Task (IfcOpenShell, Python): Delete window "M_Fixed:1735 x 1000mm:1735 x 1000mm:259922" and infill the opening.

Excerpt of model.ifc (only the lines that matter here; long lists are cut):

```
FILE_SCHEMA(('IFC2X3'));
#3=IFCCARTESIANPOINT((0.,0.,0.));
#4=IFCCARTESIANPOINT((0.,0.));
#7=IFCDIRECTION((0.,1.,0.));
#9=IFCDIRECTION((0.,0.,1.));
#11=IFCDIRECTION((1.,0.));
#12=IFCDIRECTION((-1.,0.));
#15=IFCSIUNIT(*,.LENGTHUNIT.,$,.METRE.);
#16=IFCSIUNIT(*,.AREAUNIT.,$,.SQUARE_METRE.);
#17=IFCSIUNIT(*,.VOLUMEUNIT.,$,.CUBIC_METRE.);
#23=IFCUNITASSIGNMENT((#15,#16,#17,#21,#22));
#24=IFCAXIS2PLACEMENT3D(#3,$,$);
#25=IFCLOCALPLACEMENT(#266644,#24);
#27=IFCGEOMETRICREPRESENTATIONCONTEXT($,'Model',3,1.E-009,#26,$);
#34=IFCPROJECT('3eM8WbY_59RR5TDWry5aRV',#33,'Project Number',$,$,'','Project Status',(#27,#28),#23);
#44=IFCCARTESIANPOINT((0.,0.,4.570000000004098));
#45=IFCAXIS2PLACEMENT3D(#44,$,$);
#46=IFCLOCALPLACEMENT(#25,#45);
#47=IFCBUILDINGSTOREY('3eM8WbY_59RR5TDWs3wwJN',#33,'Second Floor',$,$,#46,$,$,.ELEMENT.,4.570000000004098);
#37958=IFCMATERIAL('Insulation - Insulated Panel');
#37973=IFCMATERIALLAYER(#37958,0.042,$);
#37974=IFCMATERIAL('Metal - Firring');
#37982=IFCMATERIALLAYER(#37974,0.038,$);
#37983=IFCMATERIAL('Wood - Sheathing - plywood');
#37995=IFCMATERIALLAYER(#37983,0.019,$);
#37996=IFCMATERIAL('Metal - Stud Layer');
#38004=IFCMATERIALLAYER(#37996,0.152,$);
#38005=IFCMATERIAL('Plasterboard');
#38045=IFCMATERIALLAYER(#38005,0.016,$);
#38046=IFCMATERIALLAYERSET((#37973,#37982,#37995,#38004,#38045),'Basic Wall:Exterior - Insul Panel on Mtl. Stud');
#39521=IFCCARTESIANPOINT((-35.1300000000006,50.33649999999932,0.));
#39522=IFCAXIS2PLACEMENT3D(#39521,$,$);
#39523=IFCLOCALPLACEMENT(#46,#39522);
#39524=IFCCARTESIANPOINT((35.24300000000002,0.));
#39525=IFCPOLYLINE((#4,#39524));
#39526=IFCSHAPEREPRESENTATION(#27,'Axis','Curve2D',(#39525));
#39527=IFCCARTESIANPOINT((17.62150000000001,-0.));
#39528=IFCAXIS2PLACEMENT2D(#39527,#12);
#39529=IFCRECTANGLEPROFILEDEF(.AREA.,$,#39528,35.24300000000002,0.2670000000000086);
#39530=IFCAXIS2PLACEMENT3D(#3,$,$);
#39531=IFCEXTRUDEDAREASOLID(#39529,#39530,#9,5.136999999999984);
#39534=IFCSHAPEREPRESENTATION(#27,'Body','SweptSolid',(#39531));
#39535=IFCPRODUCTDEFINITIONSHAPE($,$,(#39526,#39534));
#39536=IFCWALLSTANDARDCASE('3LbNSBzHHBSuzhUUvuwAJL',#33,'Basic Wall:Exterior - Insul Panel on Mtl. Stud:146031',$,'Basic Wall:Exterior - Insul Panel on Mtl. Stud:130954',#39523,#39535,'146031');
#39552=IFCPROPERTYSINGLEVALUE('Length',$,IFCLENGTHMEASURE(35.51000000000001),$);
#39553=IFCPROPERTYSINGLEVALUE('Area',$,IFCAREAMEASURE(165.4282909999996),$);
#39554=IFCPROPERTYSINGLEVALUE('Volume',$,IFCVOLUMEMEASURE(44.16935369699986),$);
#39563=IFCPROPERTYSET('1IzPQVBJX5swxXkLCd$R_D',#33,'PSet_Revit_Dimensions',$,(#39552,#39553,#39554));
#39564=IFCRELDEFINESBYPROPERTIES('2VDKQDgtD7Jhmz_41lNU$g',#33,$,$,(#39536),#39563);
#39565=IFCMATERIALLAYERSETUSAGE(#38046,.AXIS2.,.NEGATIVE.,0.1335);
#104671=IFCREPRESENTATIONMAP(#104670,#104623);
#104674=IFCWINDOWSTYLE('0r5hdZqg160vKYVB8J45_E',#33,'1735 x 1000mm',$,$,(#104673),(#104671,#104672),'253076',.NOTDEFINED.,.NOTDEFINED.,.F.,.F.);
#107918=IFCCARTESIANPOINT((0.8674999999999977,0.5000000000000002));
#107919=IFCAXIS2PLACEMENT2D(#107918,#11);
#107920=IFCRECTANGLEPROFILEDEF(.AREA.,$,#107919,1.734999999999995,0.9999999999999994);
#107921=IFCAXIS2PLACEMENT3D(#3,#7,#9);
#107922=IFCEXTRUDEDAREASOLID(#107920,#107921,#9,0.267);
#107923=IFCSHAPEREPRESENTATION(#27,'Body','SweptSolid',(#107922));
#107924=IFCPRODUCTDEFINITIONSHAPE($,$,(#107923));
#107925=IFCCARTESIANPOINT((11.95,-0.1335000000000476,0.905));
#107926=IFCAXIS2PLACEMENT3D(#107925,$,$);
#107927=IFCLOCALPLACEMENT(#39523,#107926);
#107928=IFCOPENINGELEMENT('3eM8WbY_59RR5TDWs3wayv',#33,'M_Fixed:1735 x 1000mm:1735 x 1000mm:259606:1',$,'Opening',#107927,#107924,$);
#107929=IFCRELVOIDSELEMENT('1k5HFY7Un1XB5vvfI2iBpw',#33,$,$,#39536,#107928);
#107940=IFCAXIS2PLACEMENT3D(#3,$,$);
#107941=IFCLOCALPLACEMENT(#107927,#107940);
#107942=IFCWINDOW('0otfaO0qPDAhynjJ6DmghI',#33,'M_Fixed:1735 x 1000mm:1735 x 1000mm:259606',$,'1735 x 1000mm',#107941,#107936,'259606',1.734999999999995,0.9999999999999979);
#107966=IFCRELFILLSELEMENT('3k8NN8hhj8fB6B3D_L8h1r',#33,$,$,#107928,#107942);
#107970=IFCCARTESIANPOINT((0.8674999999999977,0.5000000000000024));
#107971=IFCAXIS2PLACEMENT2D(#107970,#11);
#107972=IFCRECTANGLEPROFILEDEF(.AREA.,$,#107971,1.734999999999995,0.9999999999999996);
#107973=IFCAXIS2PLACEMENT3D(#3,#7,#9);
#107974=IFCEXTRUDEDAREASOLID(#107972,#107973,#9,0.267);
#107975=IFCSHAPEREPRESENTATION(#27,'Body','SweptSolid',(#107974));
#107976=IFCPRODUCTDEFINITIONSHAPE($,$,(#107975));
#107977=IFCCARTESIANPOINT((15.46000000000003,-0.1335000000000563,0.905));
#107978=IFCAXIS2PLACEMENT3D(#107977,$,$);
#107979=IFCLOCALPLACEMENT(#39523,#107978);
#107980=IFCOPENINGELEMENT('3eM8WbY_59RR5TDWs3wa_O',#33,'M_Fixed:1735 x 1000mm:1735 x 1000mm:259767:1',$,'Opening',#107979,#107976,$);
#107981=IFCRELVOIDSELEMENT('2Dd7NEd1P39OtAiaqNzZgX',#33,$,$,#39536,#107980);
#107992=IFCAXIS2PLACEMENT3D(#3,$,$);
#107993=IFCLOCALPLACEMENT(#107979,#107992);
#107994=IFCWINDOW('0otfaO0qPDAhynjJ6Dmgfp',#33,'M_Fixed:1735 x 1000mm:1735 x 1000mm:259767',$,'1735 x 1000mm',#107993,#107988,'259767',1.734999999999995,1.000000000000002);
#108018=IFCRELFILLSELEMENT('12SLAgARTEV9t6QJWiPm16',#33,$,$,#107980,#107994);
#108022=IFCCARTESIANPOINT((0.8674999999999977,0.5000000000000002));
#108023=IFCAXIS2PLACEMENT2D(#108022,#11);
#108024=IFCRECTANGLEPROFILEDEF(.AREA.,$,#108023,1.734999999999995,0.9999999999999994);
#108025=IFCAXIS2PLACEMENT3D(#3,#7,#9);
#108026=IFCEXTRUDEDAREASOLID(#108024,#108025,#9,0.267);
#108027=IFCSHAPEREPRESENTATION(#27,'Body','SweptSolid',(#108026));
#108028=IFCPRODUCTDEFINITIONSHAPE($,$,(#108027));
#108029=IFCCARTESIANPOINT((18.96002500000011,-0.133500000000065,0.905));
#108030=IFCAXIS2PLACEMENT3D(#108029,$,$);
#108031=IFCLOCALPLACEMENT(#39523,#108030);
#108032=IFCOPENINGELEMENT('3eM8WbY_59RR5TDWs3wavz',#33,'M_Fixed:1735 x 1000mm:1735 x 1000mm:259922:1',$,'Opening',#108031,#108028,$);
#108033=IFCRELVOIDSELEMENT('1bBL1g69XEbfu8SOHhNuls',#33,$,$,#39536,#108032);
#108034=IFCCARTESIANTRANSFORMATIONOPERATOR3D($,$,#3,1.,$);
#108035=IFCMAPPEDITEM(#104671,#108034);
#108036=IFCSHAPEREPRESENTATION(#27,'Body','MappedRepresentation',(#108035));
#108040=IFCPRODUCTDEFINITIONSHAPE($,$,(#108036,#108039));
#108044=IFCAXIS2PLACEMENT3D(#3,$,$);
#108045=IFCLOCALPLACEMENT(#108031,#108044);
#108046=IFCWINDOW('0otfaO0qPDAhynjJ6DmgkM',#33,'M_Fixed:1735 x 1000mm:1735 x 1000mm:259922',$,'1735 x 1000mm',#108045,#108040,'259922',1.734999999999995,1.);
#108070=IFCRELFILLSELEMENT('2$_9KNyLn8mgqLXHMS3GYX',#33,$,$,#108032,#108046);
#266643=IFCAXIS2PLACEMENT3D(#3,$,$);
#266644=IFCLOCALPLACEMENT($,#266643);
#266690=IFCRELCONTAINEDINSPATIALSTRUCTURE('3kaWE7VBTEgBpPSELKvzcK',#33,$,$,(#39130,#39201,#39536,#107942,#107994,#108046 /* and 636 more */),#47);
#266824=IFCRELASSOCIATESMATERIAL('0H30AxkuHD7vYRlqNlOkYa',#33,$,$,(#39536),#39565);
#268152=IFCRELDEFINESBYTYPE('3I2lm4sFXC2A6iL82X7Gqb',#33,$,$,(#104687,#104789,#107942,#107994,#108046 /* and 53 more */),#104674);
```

```python
import ifcopenshell
import ifcopenshell.api.feature
import ifcopenshell.api.pset
import ifcopenshell.api.root
import ifcopenshell.geom
import ifcopenshell.util.element
import ifcopenshell.util.shape
import ifcopenshell.util.unit

model = ifcopenshell.open("model.ifc")
area_scale = ifcopenshell.util.unit.calculate_unit_scale(model, "AREAUNIT")
volume_scale = ifcopenshell.util.unit.calculate_unit_scale(model, "VOLUMEUNIT")
settings = ifcopenshell.geom.settings()


def volume(element):
    """Net volume in cubic metres, openings subtracted."""
    shape = ifcopenshell.geom.create_shape(settings, element)
    return ifcopenshell.util.shape.get_volume(shape.geometry)


window = model.by_guid("0otfaO0qPDAhynjJ6DmgkM")
opening = window.FillsVoids[0].RelatingOpeningElement
wall = opening.VoidsElements[0].RelatingBuildingElement
before = volume(wall)

ifcopenshell.api.root.remove_product(model, product=window)
ifcopenshell.api.feature.remove_feature(model, feature=opening)

after = volume(wall)
thickness = 0.267  # wall thickness in metres

# Update the wall's stored quantities.
pset = model.by_id(ifcopenshell.util.element.get_pset(wall, "PSet_Revit_Dimensions", should_inherit=False)["id"])
ifcopenshell.api.pset.edit_pset(model, pset=pset, properties={
    "Area": model.create_entity("IfcAreaMeasure", after / thickness / area_scale),
    "Volume": model.create_entity("IfcVolumeMeasure", after / volume_scale),
})

print(f"wall volume {before:.3f} -> {after:.3f} m3")

model.write("model_updated.ifc")
```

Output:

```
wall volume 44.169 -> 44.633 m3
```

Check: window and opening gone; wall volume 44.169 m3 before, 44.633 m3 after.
